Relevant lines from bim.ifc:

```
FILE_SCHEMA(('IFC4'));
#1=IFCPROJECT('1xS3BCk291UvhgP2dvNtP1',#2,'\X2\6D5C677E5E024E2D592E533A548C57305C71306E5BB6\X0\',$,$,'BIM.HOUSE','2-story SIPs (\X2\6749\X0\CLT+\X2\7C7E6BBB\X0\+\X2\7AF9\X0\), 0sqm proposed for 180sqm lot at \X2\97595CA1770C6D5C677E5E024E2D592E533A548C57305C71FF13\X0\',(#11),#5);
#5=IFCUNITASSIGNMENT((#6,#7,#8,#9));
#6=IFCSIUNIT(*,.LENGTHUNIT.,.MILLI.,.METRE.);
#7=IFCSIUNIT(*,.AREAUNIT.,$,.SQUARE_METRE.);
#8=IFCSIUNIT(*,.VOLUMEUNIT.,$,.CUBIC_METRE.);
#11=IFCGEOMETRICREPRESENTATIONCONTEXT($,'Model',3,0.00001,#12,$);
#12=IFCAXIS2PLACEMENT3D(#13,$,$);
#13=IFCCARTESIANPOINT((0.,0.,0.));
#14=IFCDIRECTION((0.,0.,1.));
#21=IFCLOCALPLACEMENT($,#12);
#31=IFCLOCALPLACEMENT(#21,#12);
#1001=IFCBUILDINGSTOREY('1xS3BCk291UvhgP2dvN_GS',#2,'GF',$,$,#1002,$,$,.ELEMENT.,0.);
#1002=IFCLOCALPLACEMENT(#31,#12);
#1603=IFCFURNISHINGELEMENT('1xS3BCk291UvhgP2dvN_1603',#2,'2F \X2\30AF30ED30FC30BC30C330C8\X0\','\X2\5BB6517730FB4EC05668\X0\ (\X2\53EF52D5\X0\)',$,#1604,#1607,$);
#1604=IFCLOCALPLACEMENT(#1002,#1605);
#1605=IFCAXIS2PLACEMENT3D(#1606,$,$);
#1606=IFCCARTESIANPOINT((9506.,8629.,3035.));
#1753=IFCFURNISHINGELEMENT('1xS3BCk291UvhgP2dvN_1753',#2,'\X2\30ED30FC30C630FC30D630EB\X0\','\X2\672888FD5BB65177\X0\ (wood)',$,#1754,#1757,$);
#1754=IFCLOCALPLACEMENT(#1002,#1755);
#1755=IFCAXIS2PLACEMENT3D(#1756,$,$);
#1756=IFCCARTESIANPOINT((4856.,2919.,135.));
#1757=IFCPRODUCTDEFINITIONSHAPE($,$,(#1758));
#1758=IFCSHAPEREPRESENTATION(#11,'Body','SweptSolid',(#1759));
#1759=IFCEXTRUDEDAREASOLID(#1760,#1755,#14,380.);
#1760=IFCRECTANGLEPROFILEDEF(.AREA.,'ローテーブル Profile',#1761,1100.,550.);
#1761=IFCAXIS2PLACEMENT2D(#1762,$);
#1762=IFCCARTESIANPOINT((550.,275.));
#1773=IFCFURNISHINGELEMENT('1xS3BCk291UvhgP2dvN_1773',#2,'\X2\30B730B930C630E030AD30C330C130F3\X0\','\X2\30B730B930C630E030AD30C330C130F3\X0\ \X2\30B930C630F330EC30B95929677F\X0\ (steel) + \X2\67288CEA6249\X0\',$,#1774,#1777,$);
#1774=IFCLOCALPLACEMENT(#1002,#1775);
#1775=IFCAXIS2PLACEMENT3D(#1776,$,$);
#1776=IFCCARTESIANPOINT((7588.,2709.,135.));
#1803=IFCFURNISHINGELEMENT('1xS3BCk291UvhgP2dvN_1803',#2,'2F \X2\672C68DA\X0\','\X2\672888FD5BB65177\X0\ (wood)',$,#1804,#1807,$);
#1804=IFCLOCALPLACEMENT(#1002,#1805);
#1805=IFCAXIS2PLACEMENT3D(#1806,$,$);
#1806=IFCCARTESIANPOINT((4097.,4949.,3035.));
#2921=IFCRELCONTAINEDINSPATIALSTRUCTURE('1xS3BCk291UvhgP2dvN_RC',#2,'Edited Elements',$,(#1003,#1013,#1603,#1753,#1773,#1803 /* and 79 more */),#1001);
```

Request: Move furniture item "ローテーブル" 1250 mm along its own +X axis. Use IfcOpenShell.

```python
import ifcopenshell
import ifcopenshell.api.geometry
import ifcopenshell.util.placement
import ifcopenshell.util.unit

model = ifcopenshell.open("bim.ifc")
unit_scale = ifcopenshell.util.unit.calculate_unit_scale(model)

item = model.by_id(1753)
matrix = ifcopenshell.util.placement.get_local_placement(item.ObjectPlacement)
matrix[:3, 3] += matrix[:3, 0] * 1.25 / unit_scale
ifcopenshell.api.geometry.edit_object_placement(model, product=item, matrix=matrix, is_si=False)

print(ifcopenshell.util.placement.get_local_placement(item.ObjectPlacement).round(3) + 0.0)

model.write("bim_updated.ifc")
```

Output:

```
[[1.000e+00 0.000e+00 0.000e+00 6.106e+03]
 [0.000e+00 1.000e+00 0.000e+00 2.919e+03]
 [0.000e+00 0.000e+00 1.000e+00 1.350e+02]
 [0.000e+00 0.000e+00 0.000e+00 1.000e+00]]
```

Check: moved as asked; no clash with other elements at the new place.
